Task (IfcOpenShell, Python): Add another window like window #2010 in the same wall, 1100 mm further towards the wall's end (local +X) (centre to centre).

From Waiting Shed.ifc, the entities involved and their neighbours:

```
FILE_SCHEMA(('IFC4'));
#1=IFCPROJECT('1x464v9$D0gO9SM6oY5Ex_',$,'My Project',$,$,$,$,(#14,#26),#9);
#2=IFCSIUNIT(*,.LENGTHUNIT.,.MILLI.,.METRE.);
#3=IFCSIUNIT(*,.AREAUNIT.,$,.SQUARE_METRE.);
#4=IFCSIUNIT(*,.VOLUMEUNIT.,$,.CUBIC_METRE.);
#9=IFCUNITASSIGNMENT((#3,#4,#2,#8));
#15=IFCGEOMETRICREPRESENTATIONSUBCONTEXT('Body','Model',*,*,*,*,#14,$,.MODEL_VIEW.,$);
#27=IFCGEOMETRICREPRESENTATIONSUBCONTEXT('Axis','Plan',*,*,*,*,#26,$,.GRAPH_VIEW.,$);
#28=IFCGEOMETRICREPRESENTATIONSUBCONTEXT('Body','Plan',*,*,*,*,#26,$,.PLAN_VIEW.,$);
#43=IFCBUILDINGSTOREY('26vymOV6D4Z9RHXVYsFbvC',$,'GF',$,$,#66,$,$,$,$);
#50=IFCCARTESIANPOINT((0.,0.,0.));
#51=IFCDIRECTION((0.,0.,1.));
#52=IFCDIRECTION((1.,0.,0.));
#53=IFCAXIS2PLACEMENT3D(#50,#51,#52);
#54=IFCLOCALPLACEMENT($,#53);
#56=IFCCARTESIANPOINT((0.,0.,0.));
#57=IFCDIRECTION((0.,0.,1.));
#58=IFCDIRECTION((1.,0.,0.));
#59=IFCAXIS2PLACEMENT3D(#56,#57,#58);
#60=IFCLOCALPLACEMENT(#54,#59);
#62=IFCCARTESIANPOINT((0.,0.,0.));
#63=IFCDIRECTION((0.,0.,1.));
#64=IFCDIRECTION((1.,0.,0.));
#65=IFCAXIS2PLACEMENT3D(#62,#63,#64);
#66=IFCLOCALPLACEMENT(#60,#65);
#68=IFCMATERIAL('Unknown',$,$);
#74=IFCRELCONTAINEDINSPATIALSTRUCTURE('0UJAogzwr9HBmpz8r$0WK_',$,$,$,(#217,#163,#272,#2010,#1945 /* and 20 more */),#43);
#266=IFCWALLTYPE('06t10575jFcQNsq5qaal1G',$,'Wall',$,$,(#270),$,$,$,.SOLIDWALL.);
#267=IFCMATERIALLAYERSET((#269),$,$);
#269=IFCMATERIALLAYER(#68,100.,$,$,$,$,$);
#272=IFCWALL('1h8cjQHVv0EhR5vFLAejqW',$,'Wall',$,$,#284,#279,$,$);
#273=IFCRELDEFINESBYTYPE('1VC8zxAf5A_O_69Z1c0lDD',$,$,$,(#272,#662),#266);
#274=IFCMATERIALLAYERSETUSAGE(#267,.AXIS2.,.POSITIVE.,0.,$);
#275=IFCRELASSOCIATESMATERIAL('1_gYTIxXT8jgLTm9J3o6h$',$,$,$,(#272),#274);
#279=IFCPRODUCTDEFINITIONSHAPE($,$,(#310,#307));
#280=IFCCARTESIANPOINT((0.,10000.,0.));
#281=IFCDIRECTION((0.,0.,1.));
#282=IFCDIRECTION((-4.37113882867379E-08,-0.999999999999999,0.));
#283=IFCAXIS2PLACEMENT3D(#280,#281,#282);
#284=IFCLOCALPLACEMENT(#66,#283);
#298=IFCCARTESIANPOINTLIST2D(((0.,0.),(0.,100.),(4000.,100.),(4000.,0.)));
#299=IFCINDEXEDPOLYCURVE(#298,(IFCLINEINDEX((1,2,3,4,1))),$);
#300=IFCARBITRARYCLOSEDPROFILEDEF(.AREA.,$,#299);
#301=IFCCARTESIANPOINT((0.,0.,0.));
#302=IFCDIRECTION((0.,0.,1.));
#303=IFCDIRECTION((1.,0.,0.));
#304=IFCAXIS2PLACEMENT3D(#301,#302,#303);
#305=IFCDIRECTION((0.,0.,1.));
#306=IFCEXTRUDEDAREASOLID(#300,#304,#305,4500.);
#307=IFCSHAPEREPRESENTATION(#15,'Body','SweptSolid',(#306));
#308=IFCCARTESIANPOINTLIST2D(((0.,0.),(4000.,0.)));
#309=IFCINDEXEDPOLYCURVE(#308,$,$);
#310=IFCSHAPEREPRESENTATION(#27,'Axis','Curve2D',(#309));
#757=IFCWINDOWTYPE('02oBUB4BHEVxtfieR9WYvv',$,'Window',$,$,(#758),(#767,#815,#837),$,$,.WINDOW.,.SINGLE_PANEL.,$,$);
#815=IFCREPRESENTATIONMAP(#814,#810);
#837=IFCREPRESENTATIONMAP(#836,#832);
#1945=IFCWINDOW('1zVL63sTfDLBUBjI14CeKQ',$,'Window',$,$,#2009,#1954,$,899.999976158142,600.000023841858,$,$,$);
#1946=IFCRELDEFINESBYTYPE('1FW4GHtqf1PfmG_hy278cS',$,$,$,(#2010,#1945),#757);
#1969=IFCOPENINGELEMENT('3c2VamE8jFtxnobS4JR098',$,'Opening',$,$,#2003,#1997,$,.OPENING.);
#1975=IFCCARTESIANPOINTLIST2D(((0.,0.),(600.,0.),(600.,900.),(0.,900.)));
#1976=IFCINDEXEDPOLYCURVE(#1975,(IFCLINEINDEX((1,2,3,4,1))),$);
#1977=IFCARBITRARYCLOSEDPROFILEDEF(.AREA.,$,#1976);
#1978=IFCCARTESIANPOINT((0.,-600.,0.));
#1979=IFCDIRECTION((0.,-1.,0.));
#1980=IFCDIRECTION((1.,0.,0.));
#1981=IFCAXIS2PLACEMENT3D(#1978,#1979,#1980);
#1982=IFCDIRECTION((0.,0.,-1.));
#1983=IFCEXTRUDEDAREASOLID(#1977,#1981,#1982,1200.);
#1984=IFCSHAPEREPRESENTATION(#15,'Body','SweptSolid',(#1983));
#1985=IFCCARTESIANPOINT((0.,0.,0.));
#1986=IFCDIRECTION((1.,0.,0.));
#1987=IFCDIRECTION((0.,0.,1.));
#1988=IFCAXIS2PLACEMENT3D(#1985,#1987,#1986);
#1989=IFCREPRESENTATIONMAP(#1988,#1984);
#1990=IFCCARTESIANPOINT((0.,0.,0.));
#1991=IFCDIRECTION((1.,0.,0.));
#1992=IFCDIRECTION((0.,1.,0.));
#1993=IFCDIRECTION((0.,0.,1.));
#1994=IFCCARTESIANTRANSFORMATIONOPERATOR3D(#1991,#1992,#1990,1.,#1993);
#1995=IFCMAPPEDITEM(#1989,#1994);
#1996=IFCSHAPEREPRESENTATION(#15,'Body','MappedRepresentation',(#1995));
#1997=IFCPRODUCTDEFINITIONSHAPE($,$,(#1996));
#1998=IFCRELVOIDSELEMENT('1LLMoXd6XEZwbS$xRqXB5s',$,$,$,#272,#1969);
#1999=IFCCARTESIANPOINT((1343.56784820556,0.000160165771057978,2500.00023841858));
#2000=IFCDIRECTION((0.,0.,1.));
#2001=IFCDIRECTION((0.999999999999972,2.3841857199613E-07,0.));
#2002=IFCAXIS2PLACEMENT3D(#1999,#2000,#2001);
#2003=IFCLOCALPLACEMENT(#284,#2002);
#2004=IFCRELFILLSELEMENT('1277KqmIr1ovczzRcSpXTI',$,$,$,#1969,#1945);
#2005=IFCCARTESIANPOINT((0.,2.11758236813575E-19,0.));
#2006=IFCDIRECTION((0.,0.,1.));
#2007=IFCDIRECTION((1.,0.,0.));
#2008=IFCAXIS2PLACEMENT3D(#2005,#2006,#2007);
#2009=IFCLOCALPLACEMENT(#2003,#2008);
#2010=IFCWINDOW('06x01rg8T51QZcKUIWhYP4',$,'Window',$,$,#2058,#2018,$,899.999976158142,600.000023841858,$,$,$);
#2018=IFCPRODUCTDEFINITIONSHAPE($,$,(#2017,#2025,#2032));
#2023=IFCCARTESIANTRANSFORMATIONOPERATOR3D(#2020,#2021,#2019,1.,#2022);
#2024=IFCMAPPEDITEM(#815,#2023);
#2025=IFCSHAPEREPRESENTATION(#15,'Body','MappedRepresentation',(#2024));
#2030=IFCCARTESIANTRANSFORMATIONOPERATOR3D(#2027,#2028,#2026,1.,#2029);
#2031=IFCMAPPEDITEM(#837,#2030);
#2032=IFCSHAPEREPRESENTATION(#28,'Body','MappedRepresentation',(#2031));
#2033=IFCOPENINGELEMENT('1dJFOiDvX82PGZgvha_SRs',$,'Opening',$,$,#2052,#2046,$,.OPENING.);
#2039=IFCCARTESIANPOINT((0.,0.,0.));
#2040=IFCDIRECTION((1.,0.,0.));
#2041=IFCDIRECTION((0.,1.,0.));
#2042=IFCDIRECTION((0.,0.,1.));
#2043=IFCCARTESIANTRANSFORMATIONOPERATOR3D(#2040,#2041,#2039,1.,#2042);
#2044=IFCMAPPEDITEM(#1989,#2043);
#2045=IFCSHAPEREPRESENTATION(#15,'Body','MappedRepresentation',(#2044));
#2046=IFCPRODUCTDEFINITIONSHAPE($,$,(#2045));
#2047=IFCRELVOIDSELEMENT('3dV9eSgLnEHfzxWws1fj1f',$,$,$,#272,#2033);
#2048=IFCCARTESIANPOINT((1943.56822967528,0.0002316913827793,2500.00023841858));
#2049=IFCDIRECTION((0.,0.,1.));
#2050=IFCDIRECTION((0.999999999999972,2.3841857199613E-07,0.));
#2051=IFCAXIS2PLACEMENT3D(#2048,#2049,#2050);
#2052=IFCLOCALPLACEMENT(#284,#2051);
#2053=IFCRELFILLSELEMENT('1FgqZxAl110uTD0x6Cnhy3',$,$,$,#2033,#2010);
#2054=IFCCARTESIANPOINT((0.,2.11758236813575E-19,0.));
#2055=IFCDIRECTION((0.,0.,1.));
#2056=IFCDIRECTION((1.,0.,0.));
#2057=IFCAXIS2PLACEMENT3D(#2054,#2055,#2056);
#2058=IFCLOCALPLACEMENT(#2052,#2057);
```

```python
import ifcopenshell
import ifcopenshell.api.feature
import ifcopenshell.api.geometry
import ifcopenshell.api.root
import ifcopenshell.geom
import ifcopenshell.util.element
import ifcopenshell.util.placement
import ifcopenshell.util.shape

model = ifcopenshell.open("Waiting Shed.ifc")
settings = ifcopenshell.geom.settings()


def volume(element):
    """Net volume in cubic metres, openings subtracted."""
    shape = ifcopenshell.geom.create_shape(settings, element)
    return ifcopenshell.util.shape.get_volume(shape.geometry)


window = model.by_guid("06x01rg8T51QZcKUIWhYP4")
opening = window.FillsVoids[0].RelatingOpeningElement
wall = opening.VoidsElements[0].RelatingBuildingElement
before = volume(wall)
shift = ifcopenshell.util.placement.get_local_placement(wall.ObjectPlacement)[:3, 0] * 1100.0

# copy_class copies the void relationship, type, container and properties, but no geometry.
new_opening = ifcopenshell.api.root.copy_class(model, product=opening)
new_opening.Representation = ifcopenshell.util.element.copy_deep(
    model, opening.Representation, exclude=["IfcGeometricRepresentationContext", "IfcRepresentationMap"]
)
new_window = ifcopenshell.api.root.copy_class(model, product=window)
new_window.Representation = ifcopenshell.util.element.copy_deep(
    model, window.Representation, exclude=["IfcGeometricRepresentationContext", "IfcRepresentationMap"]
)
ifcopenshell.api.feature.add_filling(model, opening=new_opening, element=new_window)

for old, new in ((opening, new_opening), (window, new_window)):
    matrix = ifcopenshell.util.placement.get_local_placement(old.ObjectPlacement)
    matrix[:3, 3] += shift
    ifcopenshell.api.geometry.edit_object_placement(model, product=new, matrix=matrix, is_si=False)

after = volume(wall)

print(f"wall volume {before:.3f} -> {after:.3f} m3")

model.write("Waiting Shed_v2.ifc")
```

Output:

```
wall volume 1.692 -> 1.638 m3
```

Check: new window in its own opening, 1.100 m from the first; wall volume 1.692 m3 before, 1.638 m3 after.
